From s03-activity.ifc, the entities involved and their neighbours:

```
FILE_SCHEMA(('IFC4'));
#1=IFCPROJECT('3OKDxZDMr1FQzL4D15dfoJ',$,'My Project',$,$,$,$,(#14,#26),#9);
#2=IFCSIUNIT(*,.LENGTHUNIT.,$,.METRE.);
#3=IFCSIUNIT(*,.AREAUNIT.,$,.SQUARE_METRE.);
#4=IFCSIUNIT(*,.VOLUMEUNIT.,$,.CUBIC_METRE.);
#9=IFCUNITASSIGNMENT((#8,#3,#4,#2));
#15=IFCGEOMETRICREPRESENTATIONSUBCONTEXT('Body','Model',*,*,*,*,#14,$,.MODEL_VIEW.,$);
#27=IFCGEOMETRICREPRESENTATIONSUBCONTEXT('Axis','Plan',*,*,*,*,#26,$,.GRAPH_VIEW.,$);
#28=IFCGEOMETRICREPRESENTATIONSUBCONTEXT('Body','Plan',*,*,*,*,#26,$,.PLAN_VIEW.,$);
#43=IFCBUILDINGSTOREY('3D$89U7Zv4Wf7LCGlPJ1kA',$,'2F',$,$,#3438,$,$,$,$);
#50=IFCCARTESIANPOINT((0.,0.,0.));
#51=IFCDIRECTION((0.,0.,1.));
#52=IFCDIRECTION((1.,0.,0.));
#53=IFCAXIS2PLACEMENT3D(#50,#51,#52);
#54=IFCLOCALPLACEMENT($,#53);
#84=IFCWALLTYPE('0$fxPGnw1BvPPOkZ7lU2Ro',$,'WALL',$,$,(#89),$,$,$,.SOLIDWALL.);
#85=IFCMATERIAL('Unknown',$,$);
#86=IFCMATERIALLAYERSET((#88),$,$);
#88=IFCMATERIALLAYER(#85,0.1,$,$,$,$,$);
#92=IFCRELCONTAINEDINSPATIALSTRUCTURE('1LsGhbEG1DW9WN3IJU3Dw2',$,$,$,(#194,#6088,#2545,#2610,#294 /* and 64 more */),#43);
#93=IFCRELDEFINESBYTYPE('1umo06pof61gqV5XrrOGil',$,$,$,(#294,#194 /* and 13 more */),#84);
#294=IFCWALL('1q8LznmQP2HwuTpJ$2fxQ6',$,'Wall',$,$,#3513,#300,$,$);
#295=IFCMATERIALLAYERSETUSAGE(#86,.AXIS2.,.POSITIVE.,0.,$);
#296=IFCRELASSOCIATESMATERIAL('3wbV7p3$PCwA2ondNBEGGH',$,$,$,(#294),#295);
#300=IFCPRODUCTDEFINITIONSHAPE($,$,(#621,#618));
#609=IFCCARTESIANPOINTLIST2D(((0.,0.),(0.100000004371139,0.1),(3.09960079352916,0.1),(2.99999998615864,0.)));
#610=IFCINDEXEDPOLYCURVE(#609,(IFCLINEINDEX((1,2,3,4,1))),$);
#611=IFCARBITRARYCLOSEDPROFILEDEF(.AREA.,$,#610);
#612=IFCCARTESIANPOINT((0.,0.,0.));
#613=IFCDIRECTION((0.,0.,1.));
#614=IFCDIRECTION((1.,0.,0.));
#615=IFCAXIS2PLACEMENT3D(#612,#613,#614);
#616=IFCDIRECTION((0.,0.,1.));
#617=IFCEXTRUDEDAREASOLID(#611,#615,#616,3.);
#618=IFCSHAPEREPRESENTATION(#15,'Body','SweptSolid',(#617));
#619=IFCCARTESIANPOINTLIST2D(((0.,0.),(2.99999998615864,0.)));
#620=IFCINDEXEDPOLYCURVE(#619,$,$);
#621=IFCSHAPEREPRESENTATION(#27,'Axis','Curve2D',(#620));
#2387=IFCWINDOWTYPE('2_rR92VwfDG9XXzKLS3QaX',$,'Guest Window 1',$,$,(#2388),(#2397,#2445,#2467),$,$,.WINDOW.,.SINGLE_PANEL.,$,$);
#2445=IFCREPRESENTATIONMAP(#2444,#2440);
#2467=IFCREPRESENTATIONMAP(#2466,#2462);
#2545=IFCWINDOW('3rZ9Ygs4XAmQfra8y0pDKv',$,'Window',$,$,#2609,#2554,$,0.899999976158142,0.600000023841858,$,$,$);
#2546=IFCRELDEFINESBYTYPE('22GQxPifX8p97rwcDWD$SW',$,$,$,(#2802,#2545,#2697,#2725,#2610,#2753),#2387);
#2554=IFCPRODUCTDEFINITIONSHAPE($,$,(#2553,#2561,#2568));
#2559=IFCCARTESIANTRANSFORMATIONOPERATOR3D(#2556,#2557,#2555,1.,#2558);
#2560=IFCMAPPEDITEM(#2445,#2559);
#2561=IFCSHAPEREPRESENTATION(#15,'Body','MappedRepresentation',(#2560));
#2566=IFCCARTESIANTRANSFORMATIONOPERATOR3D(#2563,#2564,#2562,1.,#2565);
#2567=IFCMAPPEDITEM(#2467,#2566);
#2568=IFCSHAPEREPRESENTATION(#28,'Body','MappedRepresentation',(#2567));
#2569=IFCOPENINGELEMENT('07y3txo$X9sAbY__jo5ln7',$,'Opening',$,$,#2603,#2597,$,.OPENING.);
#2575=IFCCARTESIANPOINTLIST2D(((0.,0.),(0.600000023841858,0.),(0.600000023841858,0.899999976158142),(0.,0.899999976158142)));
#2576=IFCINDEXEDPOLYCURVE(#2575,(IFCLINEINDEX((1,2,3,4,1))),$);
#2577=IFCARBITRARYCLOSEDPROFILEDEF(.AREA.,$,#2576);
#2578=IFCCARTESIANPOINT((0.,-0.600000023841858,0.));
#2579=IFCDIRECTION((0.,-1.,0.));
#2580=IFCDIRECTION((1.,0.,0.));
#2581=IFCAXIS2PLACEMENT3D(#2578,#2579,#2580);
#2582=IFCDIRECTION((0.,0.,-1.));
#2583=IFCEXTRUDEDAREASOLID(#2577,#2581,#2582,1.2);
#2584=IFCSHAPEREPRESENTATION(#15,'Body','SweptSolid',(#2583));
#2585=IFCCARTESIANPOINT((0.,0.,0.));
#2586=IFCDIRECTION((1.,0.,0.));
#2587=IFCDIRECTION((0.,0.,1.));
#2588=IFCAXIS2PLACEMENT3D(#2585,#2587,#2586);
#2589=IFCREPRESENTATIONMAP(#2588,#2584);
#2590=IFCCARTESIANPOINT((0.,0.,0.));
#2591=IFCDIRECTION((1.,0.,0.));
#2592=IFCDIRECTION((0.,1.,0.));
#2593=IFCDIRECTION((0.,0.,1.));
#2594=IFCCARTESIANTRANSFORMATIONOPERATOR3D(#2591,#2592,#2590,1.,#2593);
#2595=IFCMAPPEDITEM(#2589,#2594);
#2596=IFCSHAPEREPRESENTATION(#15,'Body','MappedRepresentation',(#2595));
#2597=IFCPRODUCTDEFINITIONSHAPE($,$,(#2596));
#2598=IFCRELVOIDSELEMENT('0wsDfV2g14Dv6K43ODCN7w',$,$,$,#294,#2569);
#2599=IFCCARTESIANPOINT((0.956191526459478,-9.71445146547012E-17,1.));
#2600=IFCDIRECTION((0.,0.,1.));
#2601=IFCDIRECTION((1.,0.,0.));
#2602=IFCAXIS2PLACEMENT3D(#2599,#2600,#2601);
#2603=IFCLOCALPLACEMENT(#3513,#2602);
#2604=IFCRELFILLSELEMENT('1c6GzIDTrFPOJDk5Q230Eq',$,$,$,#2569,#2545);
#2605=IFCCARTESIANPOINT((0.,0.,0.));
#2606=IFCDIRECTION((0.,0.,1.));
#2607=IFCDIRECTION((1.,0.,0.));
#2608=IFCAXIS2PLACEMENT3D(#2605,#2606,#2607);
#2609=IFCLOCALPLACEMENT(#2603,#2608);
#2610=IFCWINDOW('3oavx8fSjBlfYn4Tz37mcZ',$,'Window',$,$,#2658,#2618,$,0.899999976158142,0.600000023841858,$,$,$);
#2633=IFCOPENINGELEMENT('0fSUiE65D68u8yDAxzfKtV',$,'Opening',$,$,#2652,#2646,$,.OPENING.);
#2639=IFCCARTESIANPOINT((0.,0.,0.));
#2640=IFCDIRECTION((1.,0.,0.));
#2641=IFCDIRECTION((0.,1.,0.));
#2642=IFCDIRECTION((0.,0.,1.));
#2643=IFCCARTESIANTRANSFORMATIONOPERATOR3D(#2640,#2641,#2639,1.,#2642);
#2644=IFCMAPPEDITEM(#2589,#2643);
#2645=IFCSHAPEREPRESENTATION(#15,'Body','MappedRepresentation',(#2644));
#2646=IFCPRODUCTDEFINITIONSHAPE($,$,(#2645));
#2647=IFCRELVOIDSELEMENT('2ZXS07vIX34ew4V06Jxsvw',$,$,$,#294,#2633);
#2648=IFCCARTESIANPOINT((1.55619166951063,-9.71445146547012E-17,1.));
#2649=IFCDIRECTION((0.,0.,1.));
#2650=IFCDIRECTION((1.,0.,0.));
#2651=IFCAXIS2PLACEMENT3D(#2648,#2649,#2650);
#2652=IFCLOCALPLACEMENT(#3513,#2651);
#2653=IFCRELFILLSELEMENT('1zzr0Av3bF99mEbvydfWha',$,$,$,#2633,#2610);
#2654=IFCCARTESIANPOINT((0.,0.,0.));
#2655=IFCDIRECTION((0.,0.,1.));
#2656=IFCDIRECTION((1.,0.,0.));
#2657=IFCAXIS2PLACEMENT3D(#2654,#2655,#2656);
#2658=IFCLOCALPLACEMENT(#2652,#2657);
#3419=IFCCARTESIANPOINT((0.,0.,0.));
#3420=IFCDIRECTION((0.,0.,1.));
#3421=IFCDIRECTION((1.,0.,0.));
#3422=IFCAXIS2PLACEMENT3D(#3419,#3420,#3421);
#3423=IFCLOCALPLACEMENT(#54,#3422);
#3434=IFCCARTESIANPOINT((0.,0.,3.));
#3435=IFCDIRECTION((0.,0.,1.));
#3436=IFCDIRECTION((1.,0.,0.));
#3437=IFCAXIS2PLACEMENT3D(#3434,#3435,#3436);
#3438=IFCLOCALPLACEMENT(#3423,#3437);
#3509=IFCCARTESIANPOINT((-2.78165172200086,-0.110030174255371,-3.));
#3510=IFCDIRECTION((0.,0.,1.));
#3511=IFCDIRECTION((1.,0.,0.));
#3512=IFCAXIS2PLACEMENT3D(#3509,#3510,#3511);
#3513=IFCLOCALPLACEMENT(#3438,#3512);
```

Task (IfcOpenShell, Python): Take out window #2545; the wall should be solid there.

```python
import ifcopenshell
import ifcopenshell.api.feature
import ifcopenshell.api.root
import ifcopenshell.geom
import ifcopenshell.util.shape

model = ifcopenshell.open("s03-activity.ifc")
settings = ifcopenshell.geom.settings()


def volume(element):
    """Net volume in cubic metres, openings subtracted."""
    shape = ifcopenshell.geom.create_shape(settings, element)
    return ifcopenshell.util.shape.get_volume(shape.geometry)


window = model.by_guid("3rZ9Ygs4XAmQfra8y0pDKv")
opening = window.FillsVoids[0].RelatingOpeningElement
wall = opening.VoidsElements[0].RelatingBuildingElement
before = volume(wall)

ifcopenshell.api.root.remove_product(model, product=window)
ifcopenshell.api.feature.remove_feature(model, feature=opening)

after = volume(wall)

print(f"wall volume {before:.3f} -> {after:.3f} m3")

model.write("s03-activity_v2.ifc")
```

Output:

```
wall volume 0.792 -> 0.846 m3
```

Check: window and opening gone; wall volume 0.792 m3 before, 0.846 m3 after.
